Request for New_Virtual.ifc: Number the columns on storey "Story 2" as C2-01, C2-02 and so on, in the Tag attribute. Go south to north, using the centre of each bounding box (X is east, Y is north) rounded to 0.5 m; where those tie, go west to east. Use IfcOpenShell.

First a look at what the model holds.

```python
import ifcopenshell
import ifcopenshell.util.element
import ifcopenshell.util.placement

model = ifcopenshell.open("New_Virtual.ifc")
print(model.schema)
storey = next(s for s in model.by_type("IfcBuildingStorey") if s.Name == "Story 2")
columns = [e for e in ifcopenshell.util.element.get_decomposition(storey) if e.is_a("IfcColumn")]
for e in sorted(columns, key=lambda e: e.id()):
    origin = ifcopenshell.util.placement.get_local_placement(e.ObjectPlacement)[:3, 3]
    print(e.id(), e.Tag, e.Name, origin.round(2) + 0.0, sep=" | ")
```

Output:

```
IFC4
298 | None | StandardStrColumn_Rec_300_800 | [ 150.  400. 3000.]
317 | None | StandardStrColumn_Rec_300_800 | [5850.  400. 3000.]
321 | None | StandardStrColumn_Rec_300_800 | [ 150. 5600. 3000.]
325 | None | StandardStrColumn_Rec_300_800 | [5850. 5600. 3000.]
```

```python
import ifcopenshell
import ifcopenshell.geom
import ifcopenshell.util.element
import ifcopenshell.util.shape

model = ifcopenshell.open("New_Virtual.ifc")
settings = ifcopenshell.geom.settings()
settings.set("use-world-coords", True)


def centre(element):
    shape = ifcopenshell.geom.create_shape(settings, element)
    return ifcopenshell.util.shape.get_bbox_centroid(shape.geometry)


storey = next(s for s in model.by_type("IfcBuildingStorey") if s.Name == "Story 2")
columns = [e for e in ifcopenshell.util.element.get_decomposition(storey) if e.is_a("IfcColumn")]

# Insertion points can sit at a corner or the storey origin, so sort by the geometry (in metres).
centres = {e: centre(e) for e in columns}
columns.sort(key=lambda e: (round(centres[e][1] / 0.5), centres[e][0]))

for i, e in enumerate(columns, start=1):
    number = f"C2-{i:02d}"
    e.Tag = number
    print(e.id(), number)

model.write("New_Virtual-out.ifc")
```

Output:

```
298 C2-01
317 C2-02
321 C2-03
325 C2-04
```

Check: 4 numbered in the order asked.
